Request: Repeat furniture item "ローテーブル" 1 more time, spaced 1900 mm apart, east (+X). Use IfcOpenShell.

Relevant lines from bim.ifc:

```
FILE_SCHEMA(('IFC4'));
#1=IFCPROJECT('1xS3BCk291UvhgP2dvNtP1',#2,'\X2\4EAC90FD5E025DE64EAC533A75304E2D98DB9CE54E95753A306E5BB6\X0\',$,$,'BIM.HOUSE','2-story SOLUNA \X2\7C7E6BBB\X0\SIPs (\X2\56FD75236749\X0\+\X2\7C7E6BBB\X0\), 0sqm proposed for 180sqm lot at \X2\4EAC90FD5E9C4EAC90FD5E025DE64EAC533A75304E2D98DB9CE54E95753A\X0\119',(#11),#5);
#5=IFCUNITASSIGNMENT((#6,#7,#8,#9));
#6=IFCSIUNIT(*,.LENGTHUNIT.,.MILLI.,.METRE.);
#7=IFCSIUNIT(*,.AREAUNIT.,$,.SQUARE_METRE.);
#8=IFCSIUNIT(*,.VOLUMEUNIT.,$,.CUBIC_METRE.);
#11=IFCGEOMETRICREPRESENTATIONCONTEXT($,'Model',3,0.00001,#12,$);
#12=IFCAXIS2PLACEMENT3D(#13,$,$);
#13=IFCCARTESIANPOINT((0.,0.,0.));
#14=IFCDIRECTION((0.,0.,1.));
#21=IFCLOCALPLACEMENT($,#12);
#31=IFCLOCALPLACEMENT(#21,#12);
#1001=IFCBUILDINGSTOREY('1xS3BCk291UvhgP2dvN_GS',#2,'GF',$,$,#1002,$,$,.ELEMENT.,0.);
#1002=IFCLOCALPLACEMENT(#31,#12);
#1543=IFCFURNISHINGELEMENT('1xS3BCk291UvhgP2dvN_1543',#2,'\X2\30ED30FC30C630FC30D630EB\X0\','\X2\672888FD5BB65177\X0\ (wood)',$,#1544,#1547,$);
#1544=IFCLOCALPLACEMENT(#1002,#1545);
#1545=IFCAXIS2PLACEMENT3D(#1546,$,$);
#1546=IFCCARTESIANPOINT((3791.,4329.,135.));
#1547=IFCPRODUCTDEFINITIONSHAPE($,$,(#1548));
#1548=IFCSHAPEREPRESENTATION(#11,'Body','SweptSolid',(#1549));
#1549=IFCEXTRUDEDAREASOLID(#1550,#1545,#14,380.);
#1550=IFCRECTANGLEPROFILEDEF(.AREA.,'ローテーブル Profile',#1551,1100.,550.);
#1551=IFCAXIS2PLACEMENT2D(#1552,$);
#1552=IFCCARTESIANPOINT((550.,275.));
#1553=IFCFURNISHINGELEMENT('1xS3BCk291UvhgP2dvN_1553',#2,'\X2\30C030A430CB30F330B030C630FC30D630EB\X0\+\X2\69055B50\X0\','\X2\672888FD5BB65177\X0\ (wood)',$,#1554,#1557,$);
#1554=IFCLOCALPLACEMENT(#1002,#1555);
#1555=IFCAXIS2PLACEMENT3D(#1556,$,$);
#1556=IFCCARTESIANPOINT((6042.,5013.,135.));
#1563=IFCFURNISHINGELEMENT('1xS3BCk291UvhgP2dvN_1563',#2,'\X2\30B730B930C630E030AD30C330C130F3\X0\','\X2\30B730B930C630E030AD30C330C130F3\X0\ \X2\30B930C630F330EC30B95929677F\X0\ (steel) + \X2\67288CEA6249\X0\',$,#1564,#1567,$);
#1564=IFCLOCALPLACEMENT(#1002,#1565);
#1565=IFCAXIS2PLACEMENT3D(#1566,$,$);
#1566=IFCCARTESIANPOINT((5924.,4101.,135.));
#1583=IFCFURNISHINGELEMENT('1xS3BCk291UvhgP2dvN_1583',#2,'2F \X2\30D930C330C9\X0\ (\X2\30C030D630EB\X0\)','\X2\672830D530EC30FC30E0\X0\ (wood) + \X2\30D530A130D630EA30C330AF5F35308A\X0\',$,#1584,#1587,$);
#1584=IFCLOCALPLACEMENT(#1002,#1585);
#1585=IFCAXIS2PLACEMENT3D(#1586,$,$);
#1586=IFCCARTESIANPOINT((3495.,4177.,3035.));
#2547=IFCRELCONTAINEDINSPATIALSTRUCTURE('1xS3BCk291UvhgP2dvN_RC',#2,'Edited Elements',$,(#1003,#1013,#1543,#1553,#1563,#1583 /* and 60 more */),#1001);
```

```python
import numpy as np
import ifcopenshell
import ifcopenshell.api.geometry
import ifcopenshell.api.root
import ifcopenshell.util.element
import ifcopenshell.util.placement
import ifcopenshell.util.unit

model = ifcopenshell.open("bim.ifc")
unit_scale = ifcopenshell.util.unit.calculate_unit_scale(model)


def reuse_history(source, copy):
    """copy_class also copies each property set's owner history, people and application; keep the originals."""
    for rel in copy.IsDefinedBy:
        if rel.is_a("IfcRelDefinesByProperties") and (history := rel.RelatingPropertyDefinition.OwnerHistory):
            rel.RelatingPropertyDefinition.OwnerHistory = source.OwnerHistory
            ifcopenshell.util.element.remove_deep2(model, history)


source = model.by_guid("1xS3BCk291UvhgP2dvN_1543")
base = ifcopenshell.util.placement.get_local_placement(source.ObjectPlacement)
step = np.array([1.0, 0.0, 0.0]) * 1.9 / unit_scale

for i in range(1, 2):
    copy = ifcopenshell.api.root.copy_class(model, product=source)
    copy.Representation = ifcopenshell.util.element.copy_deep(
        model, source.Representation, exclude=["IfcGeometricRepresentationContext", "IfcRepresentationMap"]
    )
    reuse_history(source, copy)
    matrix = base.copy()
    matrix[:3, 3] += i * step
    print("added at", matrix[:3, 3].round(3) + 0.0)
    ifcopenshell.api.geometry.edit_object_placement(model, product=copy, matrix=matrix, is_si=False)

model.write("bim-out.ifc")
```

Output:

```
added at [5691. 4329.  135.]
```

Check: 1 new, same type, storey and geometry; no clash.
